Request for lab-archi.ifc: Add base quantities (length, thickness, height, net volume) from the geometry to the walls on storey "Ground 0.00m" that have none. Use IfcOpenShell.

First a look at what the model holds.

```python
import ifcopenshell
import ifcopenshell.util.element
import ifcopenshell.util.unit

model = ifcopenshell.open("lab-archi.ifc")
print(model.schema)
for unit_type in ("LENGTHUNIT", "AREAUNIT", "VOLUMEUNIT"):
    print(unit_type, ifcopenshell.util.unit.calculate_unit_scale(model, unit_type))
storey = next(s for s in model.by_type("IfcBuildingStorey") if s.Name == "Ground 0.00m")
walls = [e for e in ifcopenshell.util.element.get_decomposition(storey) if e.is_a("IfcWall")]
for e in sorted(walls, key=lambda e: e.id()):
    print(e.id(), e.is_a(), e.Name, list(ifcopenshell.util.element.get_psets(e, qtos_only=True)), sep=" | ")
```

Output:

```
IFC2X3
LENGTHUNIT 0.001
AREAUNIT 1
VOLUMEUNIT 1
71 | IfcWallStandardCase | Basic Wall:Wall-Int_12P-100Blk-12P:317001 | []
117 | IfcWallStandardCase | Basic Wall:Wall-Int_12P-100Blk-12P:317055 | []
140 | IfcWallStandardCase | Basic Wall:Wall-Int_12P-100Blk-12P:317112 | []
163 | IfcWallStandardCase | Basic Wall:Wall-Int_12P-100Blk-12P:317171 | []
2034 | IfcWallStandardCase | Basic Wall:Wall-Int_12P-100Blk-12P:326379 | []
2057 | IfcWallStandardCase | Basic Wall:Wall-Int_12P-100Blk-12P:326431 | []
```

```python
import ifcopenshell
import ifcopenshell.api.pset
import ifcopenshell.geom
import ifcopenshell.util.element
import ifcopenshell.util.shape
import ifcopenshell.util.unit

model = ifcopenshell.open("lab-archi.ifc")
unit_scale = ifcopenshell.util.unit.calculate_unit_scale(model)
volume_scale = ifcopenshell.util.unit.calculate_unit_scale(model, "VOLUMEUNIT")
settings = ifcopenshell.geom.settings()

storey = next(s for s in model.by_type("IfcBuildingStorey") if s.Name == "Ground 0.00m")
walls = [e for e in ifcopenshell.util.element.get_decomposition(storey) if e.is_a("IfcWall")]

for e in sorted(walls, key=lambda e: e.id()):
    if ifcopenshell.util.element.get_psets(e, qtos_only=True, should_inherit=False):
        continue
    # Geometry comes back in metres, in the element's own axes.
    shape = ifcopenshell.geom.create_shape(settings, e)
    values = {
        "Length": ifcopenshell.util.shape.get_x(shape.geometry) / unit_scale,
        "Width": ifcopenshell.util.shape.get_y(shape.geometry) / unit_scale,
        "Height": ifcopenshell.util.shape.get_z(shape.geometry) / unit_scale,
        "NetVolume": ifcopenshell.util.shape.get_volume(shape.geometry) / volume_scale,
    }
    qto = ifcopenshell.api.pset.add_qto(model, product=e, name="BaseQuantities")
    ifcopenshell.api.pset.edit_qto(model, qto=qto, properties=values)
    print(e.id(), {k: round(v, 3) for k, v in values.items()})

model.write("lab-archi_edited.ifc")
```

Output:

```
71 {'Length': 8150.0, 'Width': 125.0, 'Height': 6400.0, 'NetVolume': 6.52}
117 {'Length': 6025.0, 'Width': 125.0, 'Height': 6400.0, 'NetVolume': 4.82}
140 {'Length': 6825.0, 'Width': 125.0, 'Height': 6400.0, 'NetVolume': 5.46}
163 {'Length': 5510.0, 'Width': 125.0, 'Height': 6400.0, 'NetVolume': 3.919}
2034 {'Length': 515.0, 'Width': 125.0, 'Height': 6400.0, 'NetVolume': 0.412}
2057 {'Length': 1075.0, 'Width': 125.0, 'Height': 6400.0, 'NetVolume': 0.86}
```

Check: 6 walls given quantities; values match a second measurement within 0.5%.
